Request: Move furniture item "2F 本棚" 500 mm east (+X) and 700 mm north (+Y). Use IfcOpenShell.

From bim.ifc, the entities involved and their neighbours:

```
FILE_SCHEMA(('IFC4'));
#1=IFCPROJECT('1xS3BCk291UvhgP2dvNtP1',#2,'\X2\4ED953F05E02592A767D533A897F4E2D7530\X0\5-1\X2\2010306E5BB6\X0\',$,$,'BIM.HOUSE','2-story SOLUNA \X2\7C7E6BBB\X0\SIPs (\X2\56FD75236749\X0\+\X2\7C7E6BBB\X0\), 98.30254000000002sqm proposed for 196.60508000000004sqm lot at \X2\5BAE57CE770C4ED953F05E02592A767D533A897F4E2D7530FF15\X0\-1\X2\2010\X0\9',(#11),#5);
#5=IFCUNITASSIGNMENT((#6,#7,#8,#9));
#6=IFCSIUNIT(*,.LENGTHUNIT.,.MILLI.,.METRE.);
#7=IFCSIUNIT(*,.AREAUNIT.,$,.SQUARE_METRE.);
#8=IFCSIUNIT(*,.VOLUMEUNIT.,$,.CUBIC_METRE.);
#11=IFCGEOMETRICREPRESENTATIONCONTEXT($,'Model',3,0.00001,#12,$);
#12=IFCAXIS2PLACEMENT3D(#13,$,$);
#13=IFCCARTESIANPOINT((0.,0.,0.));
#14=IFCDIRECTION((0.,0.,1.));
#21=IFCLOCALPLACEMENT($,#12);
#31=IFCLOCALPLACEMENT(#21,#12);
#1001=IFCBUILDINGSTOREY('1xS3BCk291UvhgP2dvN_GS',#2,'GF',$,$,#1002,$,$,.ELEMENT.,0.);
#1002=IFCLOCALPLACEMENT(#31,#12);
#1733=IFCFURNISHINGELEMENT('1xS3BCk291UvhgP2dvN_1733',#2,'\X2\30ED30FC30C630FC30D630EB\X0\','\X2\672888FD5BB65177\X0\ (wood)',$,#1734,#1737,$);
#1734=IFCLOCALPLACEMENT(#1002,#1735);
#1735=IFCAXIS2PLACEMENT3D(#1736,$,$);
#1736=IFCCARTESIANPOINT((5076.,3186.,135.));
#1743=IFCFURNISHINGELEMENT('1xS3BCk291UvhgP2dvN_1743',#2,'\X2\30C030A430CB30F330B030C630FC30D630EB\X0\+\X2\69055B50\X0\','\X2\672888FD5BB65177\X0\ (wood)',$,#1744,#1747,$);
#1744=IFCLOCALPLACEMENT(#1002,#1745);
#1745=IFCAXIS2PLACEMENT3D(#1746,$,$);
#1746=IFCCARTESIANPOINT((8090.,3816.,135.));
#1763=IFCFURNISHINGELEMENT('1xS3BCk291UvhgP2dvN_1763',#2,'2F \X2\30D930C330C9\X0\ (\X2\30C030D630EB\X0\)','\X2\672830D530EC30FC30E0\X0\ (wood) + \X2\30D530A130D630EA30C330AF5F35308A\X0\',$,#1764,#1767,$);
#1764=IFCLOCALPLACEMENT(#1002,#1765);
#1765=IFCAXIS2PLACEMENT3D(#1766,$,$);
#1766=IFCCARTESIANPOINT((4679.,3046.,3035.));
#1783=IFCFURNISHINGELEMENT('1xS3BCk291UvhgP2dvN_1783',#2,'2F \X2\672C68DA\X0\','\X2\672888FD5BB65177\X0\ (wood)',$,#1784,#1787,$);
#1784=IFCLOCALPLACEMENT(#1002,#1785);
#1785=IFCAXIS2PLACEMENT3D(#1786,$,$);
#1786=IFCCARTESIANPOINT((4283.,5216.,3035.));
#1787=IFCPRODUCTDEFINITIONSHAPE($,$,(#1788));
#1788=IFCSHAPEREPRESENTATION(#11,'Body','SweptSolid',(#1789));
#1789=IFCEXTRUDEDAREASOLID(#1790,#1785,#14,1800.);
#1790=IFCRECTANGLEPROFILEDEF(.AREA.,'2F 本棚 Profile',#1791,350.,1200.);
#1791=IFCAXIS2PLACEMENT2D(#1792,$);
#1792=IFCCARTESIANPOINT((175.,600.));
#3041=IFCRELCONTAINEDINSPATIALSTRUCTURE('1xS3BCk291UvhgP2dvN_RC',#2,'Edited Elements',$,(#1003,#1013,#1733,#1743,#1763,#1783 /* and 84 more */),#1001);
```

```python
import ifcopenshell
import ifcopenshell.api.geometry
import ifcopenshell.util.placement
import ifcopenshell.util.unit

model = ifcopenshell.open("bim.ifc")
unit_scale = ifcopenshell.util.unit.calculate_unit_scale(model)

item = model.by_id(1783)
matrix = ifcopenshell.util.placement.get_local_placement(item.ObjectPlacement)
matrix[0, 3] += 0.5 / unit_scale
matrix[1, 3] += 0.7 / unit_scale
ifcopenshell.api.geometry.edit_object_placement(model, product=item, matrix=matrix, is_si=False)

print(ifcopenshell.util.placement.get_local_placement(item.ObjectPlacement).round(3) + 0.0)

model.write("bim_updated.ifc")
```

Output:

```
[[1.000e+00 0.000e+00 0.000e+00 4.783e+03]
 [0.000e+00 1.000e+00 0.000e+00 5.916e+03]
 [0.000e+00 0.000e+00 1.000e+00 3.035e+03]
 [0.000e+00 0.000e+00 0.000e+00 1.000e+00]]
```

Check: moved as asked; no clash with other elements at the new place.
